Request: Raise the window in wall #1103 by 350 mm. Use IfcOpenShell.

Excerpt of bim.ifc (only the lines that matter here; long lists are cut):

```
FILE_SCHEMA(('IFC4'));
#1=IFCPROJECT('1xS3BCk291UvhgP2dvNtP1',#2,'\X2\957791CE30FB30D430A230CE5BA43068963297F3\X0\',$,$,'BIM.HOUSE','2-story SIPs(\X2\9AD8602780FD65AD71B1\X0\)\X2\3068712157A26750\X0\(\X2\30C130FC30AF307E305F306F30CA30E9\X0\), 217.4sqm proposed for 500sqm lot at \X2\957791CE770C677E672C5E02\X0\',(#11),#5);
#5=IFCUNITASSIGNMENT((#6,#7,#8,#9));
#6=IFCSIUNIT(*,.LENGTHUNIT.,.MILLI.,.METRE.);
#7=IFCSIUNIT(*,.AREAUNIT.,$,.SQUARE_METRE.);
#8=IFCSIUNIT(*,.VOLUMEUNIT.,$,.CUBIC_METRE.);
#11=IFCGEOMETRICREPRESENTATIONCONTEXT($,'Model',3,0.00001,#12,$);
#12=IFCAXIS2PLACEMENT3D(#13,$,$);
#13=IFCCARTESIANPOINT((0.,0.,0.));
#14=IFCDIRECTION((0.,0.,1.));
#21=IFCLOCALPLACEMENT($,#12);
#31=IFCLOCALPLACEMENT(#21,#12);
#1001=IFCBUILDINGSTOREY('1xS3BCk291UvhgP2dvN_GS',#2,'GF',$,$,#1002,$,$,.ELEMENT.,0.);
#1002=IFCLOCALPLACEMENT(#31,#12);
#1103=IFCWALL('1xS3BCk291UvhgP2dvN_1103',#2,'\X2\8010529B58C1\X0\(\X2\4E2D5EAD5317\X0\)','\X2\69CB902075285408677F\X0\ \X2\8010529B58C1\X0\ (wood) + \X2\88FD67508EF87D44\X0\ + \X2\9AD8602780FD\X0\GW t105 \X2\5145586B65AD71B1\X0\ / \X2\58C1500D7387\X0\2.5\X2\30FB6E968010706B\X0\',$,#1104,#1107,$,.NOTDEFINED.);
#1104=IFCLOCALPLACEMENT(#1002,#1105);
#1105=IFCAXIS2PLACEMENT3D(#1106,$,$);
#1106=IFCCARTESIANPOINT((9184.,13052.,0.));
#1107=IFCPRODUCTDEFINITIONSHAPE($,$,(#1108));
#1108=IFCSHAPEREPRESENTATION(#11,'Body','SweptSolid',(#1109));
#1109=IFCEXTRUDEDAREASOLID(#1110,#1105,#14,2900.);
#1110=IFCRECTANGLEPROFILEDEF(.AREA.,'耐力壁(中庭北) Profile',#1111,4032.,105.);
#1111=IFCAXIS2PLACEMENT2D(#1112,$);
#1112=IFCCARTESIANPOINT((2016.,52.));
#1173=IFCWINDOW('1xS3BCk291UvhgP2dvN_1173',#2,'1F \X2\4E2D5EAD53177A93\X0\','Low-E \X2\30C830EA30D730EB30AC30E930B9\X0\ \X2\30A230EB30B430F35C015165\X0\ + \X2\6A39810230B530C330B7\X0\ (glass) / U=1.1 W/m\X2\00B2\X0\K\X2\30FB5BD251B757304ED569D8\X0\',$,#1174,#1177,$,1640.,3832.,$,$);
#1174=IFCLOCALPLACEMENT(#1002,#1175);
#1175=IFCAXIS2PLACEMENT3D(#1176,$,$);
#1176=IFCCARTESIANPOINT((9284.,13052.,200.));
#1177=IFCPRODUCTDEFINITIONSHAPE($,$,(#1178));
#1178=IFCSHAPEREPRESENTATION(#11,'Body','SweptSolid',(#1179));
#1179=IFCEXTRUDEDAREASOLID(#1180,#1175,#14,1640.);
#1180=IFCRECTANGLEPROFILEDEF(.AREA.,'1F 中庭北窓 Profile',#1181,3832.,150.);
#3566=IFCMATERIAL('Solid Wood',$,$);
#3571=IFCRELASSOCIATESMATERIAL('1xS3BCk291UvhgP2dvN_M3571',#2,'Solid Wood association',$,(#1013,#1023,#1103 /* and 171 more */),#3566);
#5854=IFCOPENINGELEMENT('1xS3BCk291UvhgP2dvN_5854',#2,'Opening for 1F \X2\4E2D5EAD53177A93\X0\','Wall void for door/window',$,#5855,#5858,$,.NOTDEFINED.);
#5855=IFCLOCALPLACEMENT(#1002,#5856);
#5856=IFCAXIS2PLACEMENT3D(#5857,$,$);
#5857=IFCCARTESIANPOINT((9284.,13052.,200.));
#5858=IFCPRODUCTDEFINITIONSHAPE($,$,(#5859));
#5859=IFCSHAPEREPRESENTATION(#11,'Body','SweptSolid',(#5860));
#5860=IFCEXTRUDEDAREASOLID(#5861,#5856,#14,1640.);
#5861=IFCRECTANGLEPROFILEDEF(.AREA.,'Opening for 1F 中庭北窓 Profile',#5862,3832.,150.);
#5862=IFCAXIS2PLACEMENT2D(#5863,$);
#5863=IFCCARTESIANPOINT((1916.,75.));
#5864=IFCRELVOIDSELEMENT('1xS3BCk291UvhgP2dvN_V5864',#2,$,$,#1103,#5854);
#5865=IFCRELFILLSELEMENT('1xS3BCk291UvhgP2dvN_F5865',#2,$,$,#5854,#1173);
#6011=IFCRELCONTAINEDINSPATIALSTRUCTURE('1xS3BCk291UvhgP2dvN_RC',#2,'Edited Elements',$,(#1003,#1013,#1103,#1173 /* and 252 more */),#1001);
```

```python
import numpy as np
import ifcopenshell
import ifcopenshell.api.geometry
import ifcopenshell.util.placement
import ifcopenshell.util.unit

model = ifcopenshell.open("bim.ifc")
unit_scale = ifcopenshell.util.unit.calculate_unit_scale(model)

window = model.by_guid("1xS3BCk291UvhgP2dvN_1173")
opening = window.FillsVoids[0].RelatingOpeningElement
dz = 350.0

shift = np.array([0.0, 0.0, dz])
# The window is not placed relative to its opening, so move both.
for product in (opening, window):
    matrix = ifcopenshell.util.placement.get_local_placement(product.ObjectPlacement)
    matrix[:3, 3] += shift
    ifcopenshell.api.geometry.edit_object_placement(model, product=product, matrix=matrix, is_si=False)

print(f"moved by {dz * unit_scale:+.3f} m")

model.write("bim_rev.ifc")
```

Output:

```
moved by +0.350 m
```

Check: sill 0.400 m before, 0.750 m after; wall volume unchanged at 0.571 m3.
